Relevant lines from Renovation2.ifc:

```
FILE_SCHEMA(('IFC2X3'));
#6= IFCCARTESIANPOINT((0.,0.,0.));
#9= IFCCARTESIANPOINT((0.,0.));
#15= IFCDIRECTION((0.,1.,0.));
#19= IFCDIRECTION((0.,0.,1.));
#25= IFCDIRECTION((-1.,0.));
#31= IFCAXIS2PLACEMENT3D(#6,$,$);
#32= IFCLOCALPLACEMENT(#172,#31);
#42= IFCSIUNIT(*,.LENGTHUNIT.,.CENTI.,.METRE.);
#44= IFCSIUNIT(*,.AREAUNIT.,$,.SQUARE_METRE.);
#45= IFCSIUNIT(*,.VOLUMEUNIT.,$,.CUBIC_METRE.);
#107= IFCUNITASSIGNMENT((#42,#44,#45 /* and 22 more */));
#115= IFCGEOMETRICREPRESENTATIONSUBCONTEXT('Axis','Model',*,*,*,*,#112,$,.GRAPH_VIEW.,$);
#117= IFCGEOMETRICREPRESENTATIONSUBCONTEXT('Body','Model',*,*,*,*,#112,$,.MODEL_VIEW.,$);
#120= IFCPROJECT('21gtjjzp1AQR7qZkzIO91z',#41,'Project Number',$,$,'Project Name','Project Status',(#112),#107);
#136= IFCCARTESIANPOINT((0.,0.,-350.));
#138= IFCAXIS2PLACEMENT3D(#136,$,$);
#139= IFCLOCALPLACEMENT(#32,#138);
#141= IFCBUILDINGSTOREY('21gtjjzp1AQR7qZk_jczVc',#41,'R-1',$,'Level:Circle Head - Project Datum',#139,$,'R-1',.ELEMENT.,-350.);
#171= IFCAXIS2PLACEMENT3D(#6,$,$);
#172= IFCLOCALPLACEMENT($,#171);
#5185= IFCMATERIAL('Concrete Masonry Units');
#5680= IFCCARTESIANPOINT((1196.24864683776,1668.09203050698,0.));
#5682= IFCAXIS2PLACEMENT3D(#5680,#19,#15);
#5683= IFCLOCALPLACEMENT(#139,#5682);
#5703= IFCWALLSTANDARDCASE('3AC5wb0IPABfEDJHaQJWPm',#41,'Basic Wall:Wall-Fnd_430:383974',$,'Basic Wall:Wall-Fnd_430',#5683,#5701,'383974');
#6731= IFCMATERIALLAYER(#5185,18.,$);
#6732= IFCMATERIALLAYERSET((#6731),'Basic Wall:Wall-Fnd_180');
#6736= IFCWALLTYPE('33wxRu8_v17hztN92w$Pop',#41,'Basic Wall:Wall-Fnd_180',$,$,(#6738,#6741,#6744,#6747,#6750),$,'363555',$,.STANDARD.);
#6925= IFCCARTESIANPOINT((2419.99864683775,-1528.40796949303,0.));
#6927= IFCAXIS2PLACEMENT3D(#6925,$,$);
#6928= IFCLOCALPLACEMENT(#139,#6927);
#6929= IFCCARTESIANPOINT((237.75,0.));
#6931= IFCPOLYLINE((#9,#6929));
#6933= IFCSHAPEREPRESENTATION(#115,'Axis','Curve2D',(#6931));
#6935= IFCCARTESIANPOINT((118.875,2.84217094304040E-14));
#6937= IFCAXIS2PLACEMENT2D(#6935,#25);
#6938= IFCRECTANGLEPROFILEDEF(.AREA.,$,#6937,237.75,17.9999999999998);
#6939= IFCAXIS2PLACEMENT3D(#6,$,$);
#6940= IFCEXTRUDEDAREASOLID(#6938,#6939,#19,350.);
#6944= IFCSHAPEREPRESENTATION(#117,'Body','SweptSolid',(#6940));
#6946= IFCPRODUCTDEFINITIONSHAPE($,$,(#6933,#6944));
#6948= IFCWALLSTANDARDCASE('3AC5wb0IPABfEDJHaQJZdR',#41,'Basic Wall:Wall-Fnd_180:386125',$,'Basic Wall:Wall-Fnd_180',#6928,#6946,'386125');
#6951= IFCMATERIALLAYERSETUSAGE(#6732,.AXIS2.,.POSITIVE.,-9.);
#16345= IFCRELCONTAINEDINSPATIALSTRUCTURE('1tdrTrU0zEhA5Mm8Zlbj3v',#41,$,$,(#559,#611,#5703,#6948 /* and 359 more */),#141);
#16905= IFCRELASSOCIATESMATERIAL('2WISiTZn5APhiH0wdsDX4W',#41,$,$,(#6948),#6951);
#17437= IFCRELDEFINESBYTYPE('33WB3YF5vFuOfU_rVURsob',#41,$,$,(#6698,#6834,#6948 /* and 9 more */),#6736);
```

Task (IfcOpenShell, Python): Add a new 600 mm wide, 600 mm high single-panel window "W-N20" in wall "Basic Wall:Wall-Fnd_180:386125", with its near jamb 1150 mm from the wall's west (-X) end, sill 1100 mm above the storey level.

```python
import numpy as np
import ifcopenshell
import ifcopenshell.api.feature
import ifcopenshell.api.geometry
import ifcopenshell.api.root
import ifcopenshell.api.spatial
import ifcopenshell.api.type
import ifcopenshell.geom
import ifcopenshell.util.element
import ifcopenshell.util.placement
import ifcopenshell.util.representation
import ifcopenshell.util.shape
import ifcopenshell.util.unit

model = ifcopenshell.open("Renovation2.ifc")
unit_scale = ifcopenshell.util.unit.calculate_unit_scale(model)
settings = ifcopenshell.geom.settings()


def volume(element):
    """Net volume in cubic metres, openings subtracted."""
    shape = ifcopenshell.geom.create_shape(settings, element)
    return ifcopenshell.util.shape.get_volume(shape.geometry)


wall = model.by_id(6948)
storey = ifcopenshell.util.element.get_container(wall, ifc_class="IfcBuildingStorey")
context = ifcopenshell.util.representation.get_context(model, "Model", "Body", "MODEL_VIEW")
before = volume(wall)

width, height, from_end, sill = 0.6, 0.6, 1.15, 1.1  # metres

# The wall runs along its own X axis, and the end named is its -X end.
wall_shape = ifcopenshell.geom.create_shape(settings, wall)
x, y, z = ifcopenshell.util.shape.get_vertices(wall_shape.geometry).T
start = x.min() + from_end
face, thickness = float(y.min()), float(y.max() - y.min())
wall_matrix = ifcopenshell.util.placement.get_local_placement(wall.ObjectPlacement)
level = ifcopenshell.util.placement.get_local_placement(storey.ObjectPlacement)[2, 3]


def in_wall(x, y):
    """Placement at x, y metres in the wall's axes, at sill height."""
    matrix = wall_matrix.copy()
    matrix[:, 3] = wall_matrix @ np.array([x / unit_scale, y / unit_scale, 0.0, 1.0])
    matrix[2, 3] = level + sill / unit_scale
    return matrix


# Opening: a box that overshoots both wall faces by 50 mm.
opening = ifcopenshell.api.root.create_entity(model, ifc_class="IfcOpeningElement")
box = ifcopenshell.api.geometry.add_wall_representation(
    model, context=context, length=width, height=height, thickness=thickness + 0.1
)
ifcopenshell.api.geometry.assign_representation(model, product=opening, representation=box)
ifcopenshell.api.geometry.edit_object_placement(model, product=opening, matrix=in_wall(start, face - 0.05), is_si=False)
ifcopenshell.api.feature.add_feature(model, feature=opening, element=wall)

window = ifcopenshell.api.root.create_entity(model, ifc_class="IfcWindow", name="W-N20")
window.OverallWidth, window.OverallHeight = width / unit_scale, height / unit_scale
body = ifcopenshell.api.geometry.add_window_representation(
    model,
    context=context,
    overall_width=window.OverallWidth,
    overall_height=window.OverallHeight,
    partition_type="SINGLE_PANEL",
)
ifcopenshell.api.geometry.assign_representation(model, product=window, representation=body)
ifcopenshell.api.spatial.assign_container(model, products=[window], relating_structure=storey)
fills = ifcopenshell.api.feature.add_filling(model, opening=opening, element=window)
fills.OwnerHistory = window.OwnerHistory  # required in IFC2X3

# IFC2X3 keeps the operation on the window style.
style = ifcopenshell.api.root.create_entity(model, ifc_class="IfcWindowStyle", name="W-N20")
style.OperationType, style.ConstructionType = "SINGLE_PANEL", "NOTDEFINED"
style.ParameterTakesPrecedence = style.Sizeable = False
ifcopenshell.api.type.assign_type(model, related_objects=[window], relating_type=style)

# Centre the window in the wall's thickness.
ifcopenshell.api.geometry.edit_object_placement(model, product=window, matrix=in_wall(start, face), is_si=False)
window_shape = ifcopenshell.geom.create_shape(settings, window)
depth = ifcopenshell.util.shape.get_vertices(window_shape.geometry)[:, 1]
offset = face + thickness / 2 - (depth.min() + depth.max()) / 2
ifcopenshell.api.geometry.edit_object_placement(model, product=window, matrix=in_wall(start, offset), is_si=False)

after = volume(wall)

print(f"wall volume {before:.3f} -> {after:.3f} m3")

model.write("Renovation2_edited.ifc")
```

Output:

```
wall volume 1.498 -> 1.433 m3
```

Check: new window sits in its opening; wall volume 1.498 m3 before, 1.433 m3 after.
